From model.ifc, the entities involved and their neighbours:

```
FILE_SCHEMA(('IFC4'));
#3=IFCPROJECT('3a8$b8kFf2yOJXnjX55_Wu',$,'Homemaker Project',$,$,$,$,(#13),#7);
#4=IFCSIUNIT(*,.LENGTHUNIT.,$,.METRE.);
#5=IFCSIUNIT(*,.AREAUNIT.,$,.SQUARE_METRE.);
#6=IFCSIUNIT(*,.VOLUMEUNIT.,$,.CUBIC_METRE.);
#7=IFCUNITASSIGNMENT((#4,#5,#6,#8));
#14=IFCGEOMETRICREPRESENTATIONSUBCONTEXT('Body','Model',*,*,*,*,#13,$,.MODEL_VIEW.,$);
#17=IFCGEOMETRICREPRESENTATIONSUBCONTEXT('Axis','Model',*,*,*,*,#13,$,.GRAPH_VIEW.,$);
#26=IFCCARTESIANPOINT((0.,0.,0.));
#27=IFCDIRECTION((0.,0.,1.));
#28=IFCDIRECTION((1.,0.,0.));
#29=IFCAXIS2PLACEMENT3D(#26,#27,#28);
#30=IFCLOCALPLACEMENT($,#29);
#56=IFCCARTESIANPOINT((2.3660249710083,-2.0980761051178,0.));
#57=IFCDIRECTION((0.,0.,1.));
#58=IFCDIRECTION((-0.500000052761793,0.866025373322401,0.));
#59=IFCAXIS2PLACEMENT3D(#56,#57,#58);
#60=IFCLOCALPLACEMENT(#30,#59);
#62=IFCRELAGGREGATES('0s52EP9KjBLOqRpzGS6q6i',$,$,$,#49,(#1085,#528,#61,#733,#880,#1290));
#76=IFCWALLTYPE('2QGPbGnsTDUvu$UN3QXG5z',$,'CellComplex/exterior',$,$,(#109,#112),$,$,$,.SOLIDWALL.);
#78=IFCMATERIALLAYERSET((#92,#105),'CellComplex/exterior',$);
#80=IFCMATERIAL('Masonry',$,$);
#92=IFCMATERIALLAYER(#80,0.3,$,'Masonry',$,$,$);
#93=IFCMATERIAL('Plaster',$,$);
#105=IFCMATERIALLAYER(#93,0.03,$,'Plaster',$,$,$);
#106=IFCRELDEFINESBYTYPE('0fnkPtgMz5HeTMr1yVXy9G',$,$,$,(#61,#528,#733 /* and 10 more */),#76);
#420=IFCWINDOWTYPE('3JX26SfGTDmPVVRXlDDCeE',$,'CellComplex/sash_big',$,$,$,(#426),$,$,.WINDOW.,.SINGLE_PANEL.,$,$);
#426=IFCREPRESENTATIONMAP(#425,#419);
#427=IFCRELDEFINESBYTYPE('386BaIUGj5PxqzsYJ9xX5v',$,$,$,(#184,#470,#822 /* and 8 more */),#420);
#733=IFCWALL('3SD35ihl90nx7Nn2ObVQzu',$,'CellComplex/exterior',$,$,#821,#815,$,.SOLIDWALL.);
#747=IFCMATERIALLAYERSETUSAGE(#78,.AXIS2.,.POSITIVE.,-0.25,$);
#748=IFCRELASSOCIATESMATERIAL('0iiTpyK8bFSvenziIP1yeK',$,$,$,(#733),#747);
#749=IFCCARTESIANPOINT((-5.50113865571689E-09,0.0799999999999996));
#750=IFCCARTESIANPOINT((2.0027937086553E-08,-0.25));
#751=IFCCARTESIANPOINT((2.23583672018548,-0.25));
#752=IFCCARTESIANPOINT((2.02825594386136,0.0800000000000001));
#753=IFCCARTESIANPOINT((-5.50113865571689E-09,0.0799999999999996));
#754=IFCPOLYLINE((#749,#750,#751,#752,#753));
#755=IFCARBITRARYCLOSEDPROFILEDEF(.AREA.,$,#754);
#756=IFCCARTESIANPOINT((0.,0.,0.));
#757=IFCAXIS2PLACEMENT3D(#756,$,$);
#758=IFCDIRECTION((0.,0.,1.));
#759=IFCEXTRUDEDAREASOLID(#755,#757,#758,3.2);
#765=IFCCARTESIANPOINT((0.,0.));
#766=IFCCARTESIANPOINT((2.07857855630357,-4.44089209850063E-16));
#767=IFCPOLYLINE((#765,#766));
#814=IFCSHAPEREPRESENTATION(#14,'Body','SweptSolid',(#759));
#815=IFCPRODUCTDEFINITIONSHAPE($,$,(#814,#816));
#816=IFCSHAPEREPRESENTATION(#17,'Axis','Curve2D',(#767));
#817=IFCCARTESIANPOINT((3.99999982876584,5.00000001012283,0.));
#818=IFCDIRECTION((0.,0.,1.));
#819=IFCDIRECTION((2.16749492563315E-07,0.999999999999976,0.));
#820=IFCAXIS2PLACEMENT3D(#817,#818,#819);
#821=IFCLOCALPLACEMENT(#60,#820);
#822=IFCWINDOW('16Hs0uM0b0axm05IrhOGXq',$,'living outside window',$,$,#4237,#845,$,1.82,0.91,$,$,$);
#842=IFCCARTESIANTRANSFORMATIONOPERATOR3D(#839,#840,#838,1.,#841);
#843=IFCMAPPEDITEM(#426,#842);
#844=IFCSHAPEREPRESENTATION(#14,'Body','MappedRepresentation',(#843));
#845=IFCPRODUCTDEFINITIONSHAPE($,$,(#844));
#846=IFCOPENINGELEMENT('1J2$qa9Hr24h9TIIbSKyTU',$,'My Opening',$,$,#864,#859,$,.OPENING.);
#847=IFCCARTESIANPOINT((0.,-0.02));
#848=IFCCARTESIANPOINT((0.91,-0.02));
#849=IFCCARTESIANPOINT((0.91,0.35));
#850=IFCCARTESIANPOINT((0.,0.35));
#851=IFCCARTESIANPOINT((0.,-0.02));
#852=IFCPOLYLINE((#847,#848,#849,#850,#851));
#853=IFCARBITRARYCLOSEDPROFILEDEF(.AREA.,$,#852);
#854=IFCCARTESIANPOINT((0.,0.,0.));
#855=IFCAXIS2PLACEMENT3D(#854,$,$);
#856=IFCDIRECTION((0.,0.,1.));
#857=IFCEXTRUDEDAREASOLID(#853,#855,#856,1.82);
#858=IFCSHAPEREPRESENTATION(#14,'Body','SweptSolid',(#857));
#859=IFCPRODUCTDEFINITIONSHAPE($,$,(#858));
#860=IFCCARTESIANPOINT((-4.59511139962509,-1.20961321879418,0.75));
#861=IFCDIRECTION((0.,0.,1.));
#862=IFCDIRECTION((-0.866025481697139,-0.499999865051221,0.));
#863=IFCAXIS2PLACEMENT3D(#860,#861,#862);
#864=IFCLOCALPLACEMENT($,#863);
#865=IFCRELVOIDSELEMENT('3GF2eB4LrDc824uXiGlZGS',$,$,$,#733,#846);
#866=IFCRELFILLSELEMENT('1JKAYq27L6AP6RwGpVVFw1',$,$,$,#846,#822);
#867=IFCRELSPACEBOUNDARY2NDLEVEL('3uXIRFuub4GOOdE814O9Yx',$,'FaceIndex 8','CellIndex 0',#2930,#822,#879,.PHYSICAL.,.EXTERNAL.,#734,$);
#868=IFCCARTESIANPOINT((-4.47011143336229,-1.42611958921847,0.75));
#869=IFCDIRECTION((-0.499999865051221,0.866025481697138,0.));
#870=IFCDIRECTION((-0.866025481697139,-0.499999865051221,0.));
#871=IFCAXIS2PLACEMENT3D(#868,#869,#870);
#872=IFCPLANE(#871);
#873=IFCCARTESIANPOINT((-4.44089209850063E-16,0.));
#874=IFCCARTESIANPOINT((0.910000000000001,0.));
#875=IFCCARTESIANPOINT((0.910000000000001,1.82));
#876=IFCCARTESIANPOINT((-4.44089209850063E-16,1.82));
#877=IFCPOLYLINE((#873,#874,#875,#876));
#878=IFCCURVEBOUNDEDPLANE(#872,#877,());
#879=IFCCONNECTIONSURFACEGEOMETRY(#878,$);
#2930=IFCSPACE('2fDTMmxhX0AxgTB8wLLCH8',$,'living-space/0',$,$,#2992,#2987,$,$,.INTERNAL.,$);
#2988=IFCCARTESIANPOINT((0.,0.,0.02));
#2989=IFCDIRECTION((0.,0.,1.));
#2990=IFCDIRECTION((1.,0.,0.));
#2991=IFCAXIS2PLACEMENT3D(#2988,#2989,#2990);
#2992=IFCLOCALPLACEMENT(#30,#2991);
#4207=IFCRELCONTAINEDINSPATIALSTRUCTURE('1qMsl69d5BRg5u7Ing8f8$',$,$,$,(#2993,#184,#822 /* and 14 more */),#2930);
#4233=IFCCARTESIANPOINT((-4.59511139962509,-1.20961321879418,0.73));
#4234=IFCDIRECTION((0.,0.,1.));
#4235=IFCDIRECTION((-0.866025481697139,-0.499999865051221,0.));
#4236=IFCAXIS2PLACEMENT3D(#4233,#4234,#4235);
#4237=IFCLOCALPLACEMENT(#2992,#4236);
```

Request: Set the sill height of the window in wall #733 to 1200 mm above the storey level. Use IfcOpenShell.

```python
import numpy as np
import ifcopenshell
import ifcopenshell.api.geometry
import ifcopenshell.geom
import ifcopenshell.util.element
import ifcopenshell.util.placement
import ifcopenshell.util.shape
import ifcopenshell.util.unit

model = ifcopenshell.open("model.ifc")
unit_scale = ifcopenshell.util.unit.calculate_unit_scale(model)

window = model.by_id(822)
opening = window.FillsVoids[0].RelatingOpeningElement
storey = ifcopenshell.util.element.get_container(window, ifc_class="IfcBuildingStorey")
level = ifcopenshell.util.placement.get_local_placement(storey.ObjectPlacement)[2, 3]

# The opening's origin need not be at the sill, so measure its lowest point.
shape = ifcopenshell.geom.create_shape(ifcopenshell.geom.settings(), opening)
bottom = ifcopenshell.util.shape.get_shape_bottom_elevation(shape, shape.geometry) / unit_scale
dz = level + 1.2 / unit_scale - bottom

shift = np.array([0.0, 0.0, dz])
# The window is not placed relative to its opening, so move both.
for product in (opening, window):
    matrix = ifcopenshell.util.placement.get_local_placement(product.ObjectPlacement)
    matrix[:3, 3] += shift
    ifcopenshell.api.geometry.edit_object_placement(model, product=product, matrix=matrix, is_si=False)

# Space boundary surfaces are stored in each space's coordinates; move them too.
for rel in window.ProvidesBoundaries:
    if not rel.ConnectionGeometry:
        continue
    surface = rel.ConnectionGeometry.SurfaceOnRelatingElement.BasisSurface
    space_matrix = ifcopenshell.util.placement.get_local_placement(rel.RelatingSpace.ObjectPlacement)
    point = np.array(surface.Position.Location.Coordinates) + space_matrix[:3, :3].T @ shift
    surface.Position = model.createIfcAxis2Placement3D(
        model.createIfcCartesianPoint(point.tolist()), surface.Position.Axis, surface.Position.RefDirection
    )

print(f"moved by {dz * unit_scale:+.3f} m")

model.write("model-out.ifc")
```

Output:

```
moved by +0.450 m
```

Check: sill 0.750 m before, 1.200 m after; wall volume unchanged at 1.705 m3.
